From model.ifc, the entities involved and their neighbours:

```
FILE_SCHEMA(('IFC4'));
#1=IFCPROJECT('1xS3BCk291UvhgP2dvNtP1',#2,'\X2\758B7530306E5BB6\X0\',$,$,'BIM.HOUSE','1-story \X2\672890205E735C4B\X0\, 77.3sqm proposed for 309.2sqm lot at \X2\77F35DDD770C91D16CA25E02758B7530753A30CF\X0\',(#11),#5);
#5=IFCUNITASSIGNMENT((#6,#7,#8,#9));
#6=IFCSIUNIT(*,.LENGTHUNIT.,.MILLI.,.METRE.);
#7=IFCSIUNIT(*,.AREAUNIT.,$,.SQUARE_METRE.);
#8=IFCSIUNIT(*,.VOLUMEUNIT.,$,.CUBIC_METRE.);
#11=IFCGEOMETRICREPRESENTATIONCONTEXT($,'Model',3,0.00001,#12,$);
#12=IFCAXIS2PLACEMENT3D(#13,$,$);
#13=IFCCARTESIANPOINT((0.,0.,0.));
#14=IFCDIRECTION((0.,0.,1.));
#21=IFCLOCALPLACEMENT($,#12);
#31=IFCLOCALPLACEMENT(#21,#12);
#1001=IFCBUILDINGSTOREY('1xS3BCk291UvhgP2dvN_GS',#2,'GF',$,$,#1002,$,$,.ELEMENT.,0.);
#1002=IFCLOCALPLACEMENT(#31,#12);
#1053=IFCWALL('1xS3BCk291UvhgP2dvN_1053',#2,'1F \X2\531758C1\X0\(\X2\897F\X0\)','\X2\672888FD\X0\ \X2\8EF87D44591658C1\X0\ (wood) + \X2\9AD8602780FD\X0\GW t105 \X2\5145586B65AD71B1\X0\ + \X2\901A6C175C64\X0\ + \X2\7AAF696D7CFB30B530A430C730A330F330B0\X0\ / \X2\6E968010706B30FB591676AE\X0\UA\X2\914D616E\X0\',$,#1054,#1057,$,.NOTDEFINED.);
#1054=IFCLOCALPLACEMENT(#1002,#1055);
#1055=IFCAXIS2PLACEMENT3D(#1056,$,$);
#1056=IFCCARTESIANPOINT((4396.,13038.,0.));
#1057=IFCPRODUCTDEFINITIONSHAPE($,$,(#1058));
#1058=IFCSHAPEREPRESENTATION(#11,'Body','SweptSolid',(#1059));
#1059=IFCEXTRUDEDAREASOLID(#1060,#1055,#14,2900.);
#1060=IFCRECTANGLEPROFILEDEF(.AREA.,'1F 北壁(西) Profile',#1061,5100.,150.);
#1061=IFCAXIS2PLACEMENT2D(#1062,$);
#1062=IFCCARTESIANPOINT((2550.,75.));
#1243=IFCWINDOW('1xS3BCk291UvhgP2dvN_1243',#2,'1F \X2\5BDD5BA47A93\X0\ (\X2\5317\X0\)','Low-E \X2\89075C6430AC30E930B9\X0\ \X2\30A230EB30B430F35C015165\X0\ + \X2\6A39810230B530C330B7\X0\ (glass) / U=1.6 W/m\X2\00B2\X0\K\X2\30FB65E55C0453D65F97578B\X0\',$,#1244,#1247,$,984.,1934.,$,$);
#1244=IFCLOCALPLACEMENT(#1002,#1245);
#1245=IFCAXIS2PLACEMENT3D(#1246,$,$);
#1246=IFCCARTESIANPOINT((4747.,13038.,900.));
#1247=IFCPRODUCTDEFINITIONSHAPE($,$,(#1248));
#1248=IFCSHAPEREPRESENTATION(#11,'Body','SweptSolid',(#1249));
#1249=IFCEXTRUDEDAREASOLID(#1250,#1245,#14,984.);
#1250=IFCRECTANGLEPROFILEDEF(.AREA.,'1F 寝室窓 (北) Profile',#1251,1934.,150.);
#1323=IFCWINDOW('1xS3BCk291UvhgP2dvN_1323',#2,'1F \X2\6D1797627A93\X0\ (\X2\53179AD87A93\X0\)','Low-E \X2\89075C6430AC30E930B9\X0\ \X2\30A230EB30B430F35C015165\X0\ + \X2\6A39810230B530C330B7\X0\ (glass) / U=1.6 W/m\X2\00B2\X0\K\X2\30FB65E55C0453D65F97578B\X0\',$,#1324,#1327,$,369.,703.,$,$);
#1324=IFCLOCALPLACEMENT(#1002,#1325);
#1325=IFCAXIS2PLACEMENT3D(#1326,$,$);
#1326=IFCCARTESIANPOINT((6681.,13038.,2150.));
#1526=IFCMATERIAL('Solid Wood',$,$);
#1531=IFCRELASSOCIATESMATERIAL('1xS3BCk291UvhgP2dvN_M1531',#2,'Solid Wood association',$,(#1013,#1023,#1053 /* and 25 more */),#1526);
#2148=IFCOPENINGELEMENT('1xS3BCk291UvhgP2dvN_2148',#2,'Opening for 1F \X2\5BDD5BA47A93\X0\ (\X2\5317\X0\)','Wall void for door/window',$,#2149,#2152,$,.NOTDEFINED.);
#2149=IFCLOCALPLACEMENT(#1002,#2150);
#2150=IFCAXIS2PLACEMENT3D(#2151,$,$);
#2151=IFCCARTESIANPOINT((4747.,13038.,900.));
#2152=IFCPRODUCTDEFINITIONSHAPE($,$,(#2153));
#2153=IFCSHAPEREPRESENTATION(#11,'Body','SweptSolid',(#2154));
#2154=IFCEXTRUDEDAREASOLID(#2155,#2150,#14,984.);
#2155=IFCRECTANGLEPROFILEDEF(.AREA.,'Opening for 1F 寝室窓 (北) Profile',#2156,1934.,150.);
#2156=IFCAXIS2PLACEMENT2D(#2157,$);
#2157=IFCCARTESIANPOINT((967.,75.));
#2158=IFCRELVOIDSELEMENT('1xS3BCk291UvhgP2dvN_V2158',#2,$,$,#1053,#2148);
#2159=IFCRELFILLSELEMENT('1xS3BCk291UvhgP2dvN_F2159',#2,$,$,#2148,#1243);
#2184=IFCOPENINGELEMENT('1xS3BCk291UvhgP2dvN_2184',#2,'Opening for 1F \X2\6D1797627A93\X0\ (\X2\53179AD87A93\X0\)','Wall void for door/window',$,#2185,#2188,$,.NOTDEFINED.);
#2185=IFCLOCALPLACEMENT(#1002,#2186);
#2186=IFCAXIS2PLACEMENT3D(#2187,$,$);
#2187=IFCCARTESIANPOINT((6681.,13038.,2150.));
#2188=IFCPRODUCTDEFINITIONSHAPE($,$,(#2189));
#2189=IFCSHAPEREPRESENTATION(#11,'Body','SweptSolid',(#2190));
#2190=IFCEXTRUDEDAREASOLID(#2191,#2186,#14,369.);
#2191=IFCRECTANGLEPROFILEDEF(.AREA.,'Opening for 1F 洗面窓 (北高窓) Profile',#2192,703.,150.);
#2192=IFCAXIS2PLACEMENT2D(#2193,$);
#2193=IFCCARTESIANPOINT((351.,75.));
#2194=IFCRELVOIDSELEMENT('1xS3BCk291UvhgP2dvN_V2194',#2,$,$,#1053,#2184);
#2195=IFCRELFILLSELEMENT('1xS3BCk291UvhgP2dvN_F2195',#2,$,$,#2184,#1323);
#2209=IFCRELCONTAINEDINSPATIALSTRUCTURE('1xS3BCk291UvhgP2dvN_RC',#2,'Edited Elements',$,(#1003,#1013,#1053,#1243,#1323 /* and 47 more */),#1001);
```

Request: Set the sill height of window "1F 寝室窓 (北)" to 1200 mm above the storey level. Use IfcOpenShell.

```python
import numpy as np
import ifcopenshell
import ifcopenshell.api.geometry
import ifcopenshell.geom
import ifcopenshell.util.element
import ifcopenshell.util.placement
import ifcopenshell.util.shape
import ifcopenshell.util.unit

model = ifcopenshell.open("model.ifc")
unit_scale = ifcopenshell.util.unit.calculate_unit_scale(model)

window = model.by_guid("1xS3BCk291UvhgP2dvN_1243")
opening = window.FillsVoids[0].RelatingOpeningElement
storey = ifcopenshell.util.element.get_container(window, ifc_class="IfcBuildingStorey")
level = ifcopenshell.util.placement.get_local_placement(storey.ObjectPlacement)[2, 3]

# The opening's origin need not be at the sill, so measure its lowest point.
shape = ifcopenshell.geom.create_shape(ifcopenshell.geom.settings(), opening)
bottom = ifcopenshell.util.shape.get_shape_bottom_elevation(shape, shape.geometry) / unit_scale
dz = level + 1200.0 - bottom

shift = np.array([0.0, 0.0, dz])
# The window is not placed relative to its opening, so move both.
for product in (opening, window):
    matrix = ifcopenshell.util.placement.get_local_placement(product.ObjectPlacement)
    matrix[:3, 3] += shift
    ifcopenshell.api.geometry.edit_object_placement(model, product=product, matrix=matrix, is_si=False)

print(f"moved by {dz * unit_scale:+.3f} m")

model.write("model-out.ifc")
```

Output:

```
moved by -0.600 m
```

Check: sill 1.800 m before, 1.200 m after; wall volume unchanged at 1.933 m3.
